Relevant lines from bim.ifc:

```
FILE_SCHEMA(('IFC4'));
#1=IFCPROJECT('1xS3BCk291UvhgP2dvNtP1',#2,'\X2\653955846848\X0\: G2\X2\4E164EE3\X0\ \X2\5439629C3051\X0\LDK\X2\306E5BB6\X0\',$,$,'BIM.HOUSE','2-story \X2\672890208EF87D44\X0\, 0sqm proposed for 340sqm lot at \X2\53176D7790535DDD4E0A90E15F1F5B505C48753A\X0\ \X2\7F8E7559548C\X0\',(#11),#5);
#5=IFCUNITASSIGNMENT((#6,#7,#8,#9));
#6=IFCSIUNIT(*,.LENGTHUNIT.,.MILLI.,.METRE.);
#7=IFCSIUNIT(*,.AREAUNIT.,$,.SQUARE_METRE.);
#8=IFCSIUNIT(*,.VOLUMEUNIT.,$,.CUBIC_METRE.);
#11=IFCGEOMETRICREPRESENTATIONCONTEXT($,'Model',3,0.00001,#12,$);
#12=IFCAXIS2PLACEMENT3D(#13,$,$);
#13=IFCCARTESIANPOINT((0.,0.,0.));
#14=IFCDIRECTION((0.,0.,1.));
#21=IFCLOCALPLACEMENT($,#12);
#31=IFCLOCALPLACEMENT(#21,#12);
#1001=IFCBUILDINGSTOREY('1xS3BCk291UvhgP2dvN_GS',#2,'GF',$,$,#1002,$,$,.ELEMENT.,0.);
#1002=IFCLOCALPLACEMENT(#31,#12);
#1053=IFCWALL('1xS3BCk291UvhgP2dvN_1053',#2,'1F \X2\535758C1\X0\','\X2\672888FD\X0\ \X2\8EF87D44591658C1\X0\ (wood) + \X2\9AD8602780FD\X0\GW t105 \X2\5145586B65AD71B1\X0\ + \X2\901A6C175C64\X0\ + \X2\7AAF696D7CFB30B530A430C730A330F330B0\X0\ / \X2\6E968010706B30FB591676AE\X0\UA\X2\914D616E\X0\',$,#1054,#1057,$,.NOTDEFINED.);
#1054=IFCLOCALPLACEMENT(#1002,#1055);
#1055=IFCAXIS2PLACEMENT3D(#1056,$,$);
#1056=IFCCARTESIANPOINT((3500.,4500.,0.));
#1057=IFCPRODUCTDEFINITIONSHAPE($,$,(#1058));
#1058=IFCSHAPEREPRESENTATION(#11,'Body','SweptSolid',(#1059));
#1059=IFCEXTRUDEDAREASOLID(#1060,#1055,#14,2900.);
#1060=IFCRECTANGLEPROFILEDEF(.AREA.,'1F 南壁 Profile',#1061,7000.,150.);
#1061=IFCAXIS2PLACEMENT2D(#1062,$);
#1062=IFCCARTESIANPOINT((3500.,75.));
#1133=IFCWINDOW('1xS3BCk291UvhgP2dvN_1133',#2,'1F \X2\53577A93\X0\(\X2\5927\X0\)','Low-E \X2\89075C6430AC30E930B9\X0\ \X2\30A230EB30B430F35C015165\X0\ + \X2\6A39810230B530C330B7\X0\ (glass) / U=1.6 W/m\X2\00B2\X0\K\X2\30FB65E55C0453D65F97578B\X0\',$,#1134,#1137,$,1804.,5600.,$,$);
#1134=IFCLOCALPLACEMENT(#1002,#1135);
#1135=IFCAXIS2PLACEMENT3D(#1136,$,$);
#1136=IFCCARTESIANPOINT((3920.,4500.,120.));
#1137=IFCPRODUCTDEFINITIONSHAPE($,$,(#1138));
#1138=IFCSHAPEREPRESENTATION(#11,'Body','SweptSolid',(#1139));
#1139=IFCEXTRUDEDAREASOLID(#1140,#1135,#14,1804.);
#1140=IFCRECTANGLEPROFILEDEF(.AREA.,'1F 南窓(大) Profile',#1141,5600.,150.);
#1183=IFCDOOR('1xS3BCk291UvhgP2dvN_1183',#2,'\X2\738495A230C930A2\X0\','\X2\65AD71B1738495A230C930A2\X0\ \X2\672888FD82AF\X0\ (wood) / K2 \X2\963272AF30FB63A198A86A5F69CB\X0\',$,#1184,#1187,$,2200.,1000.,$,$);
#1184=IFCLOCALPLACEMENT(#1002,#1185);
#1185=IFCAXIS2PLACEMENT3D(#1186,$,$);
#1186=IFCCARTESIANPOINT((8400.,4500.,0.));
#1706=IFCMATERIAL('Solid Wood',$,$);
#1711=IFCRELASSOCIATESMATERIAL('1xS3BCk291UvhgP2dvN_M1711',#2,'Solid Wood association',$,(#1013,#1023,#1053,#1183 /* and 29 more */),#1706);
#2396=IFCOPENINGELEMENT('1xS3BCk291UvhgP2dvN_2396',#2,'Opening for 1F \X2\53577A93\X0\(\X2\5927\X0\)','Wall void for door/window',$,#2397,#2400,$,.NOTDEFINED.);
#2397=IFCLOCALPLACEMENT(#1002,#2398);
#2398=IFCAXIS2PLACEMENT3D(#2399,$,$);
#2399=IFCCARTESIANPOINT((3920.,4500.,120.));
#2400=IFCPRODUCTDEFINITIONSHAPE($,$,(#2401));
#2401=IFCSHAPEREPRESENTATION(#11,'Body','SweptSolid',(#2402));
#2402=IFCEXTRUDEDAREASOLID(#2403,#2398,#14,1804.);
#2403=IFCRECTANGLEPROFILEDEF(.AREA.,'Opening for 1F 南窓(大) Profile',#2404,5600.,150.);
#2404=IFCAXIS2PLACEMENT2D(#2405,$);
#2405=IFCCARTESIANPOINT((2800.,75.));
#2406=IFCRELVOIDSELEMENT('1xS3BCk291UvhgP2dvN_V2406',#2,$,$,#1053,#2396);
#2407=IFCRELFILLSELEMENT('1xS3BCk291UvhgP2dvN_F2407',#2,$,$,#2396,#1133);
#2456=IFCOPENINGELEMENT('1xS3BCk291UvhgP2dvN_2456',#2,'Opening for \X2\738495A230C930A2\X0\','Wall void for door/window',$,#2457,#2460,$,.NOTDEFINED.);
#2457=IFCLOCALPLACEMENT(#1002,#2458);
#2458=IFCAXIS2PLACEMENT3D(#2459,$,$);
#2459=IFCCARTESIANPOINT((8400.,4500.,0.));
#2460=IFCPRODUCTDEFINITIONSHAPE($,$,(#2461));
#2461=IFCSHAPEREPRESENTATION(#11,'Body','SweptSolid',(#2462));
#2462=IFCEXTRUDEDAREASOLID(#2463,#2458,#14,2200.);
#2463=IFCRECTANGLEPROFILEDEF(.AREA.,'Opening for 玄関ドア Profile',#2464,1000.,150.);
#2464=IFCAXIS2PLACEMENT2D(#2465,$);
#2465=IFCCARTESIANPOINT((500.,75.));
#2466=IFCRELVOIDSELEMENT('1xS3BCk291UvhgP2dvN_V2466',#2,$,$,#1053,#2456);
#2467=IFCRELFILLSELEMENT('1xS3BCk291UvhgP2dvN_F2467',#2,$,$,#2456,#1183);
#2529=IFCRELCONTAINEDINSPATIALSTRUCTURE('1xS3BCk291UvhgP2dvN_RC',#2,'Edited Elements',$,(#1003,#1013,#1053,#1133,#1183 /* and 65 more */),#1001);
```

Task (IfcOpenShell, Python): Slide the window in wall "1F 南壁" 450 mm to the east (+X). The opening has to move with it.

```python
import ifcopenshell
import ifcopenshell.api.geometry
import ifcopenshell.util.placement

model = ifcopenshell.open("bim.ifc")

window = model.by_guid("1xS3BCk291UvhgP2dvN_1133")
opening = window.FillsVoids[0].RelatingOpeningElement
wall = opening.VoidsElements[0].RelatingBuildingElement

wall_matrix = ifcopenshell.util.placement.get_local_placement(wall.ObjectPlacement)
shift = wall_matrix[:3, 0] * 450.0
before = ifcopenshell.util.placement.get_local_placement(window.ObjectPlacement)[:3, 3].copy()

# The window is not placed relative to its opening, so move both.
for product in (opening, window):
    matrix = ifcopenshell.util.placement.get_local_placement(product.ObjectPlacement)
    matrix[:3, 3] += shift
    ifcopenshell.api.geometry.edit_object_placement(model, product=product, matrix=matrix, is_si=False)

after = ifcopenshell.util.placement.get_local_placement(window.ObjectPlacement)[:3, 3]
print("window moved by", (after - before).round(3) + 0.0)

model.write("bim_v2.ifc")
```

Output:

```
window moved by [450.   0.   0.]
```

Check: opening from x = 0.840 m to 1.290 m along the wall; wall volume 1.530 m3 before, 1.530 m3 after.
